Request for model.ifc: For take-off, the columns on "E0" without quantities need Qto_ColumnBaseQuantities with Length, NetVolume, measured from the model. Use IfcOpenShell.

First a look at what the model holds.

```python
import ifcopenshell
import ifcopenshell.util.element
import ifcopenshell.util.unit

model = ifcopenshell.open("model.ifc")
print(model.schema)
for unit_type in ("LENGTHUNIT", "AREAUNIT", "VOLUMEUNIT"):
    print(unit_type, ifcopenshell.util.unit.calculate_unit_scale(model, unit_type))
storey = next(s for s in model.by_type("IfcBuildingStorey") if s.Name == "E0")
columns = [e for e in ifcopenshell.util.element.get_decomposition(storey) if e.is_a("IfcColumn")]
for e in sorted(columns, key=lambda e: e.id()):
    print(e.id(), e.is_a(), e.Name, list(ifcopenshell.util.element.get_psets(e, qtos_only=True)), sep=" | ")
```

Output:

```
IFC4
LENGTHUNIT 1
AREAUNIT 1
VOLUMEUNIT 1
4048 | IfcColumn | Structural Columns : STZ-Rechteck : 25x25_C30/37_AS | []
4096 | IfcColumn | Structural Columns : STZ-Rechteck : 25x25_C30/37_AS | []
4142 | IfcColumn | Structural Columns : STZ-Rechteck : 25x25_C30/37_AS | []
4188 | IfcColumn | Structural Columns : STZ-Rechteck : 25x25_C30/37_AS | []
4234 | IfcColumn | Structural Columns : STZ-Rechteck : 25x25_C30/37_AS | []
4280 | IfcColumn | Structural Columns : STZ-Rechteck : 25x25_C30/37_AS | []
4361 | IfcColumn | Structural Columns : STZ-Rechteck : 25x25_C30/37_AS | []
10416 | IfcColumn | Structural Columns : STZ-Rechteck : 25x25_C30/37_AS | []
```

```python
import ifcopenshell
import ifcopenshell.api.pset
import ifcopenshell.geom
import ifcopenshell.util.element
import ifcopenshell.util.shape
import ifcopenshell.util.unit

model = ifcopenshell.open("model.ifc")
unit_scale = ifcopenshell.util.unit.calculate_unit_scale(model)
volume_scale = ifcopenshell.util.unit.calculate_unit_scale(model, "VOLUMEUNIT")
settings = ifcopenshell.geom.settings()

storey = next(s for s in model.by_type("IfcBuildingStorey") if s.Name == "E0")
columns = [e for e in ifcopenshell.util.element.get_decomposition(storey) if e.is_a("IfcColumn")]

for e in sorted(columns, key=lambda e: e.id()):
    if ifcopenshell.util.element.get_psets(e, qtos_only=True, should_inherit=False):
        continue
    # Geometry comes back in metres, in the element's own axes.
    shape = ifcopenshell.geom.create_shape(settings, e)
    values = {
        "Length": ifcopenshell.util.shape.get_z(shape.geometry) / unit_scale,
        "NetVolume": ifcopenshell.util.shape.get_volume(shape.geometry) / volume_scale,
    }
    qto = ifcopenshell.api.pset.add_qto(model, product=e, name="Qto_ColumnBaseQuantities")
    ifcopenshell.api.pset.edit_qto(model, qto=qto, properties=values)
    print(e.id(), {k: round(v, 3) for k, v in values.items()})

model.write("model_rev.ifc")
```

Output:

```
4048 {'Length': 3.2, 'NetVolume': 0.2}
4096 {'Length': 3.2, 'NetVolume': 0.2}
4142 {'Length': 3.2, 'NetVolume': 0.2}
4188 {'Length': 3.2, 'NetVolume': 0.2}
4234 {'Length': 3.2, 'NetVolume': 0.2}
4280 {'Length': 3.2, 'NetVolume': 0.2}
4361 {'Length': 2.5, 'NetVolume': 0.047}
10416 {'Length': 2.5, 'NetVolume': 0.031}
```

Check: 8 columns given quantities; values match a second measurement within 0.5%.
